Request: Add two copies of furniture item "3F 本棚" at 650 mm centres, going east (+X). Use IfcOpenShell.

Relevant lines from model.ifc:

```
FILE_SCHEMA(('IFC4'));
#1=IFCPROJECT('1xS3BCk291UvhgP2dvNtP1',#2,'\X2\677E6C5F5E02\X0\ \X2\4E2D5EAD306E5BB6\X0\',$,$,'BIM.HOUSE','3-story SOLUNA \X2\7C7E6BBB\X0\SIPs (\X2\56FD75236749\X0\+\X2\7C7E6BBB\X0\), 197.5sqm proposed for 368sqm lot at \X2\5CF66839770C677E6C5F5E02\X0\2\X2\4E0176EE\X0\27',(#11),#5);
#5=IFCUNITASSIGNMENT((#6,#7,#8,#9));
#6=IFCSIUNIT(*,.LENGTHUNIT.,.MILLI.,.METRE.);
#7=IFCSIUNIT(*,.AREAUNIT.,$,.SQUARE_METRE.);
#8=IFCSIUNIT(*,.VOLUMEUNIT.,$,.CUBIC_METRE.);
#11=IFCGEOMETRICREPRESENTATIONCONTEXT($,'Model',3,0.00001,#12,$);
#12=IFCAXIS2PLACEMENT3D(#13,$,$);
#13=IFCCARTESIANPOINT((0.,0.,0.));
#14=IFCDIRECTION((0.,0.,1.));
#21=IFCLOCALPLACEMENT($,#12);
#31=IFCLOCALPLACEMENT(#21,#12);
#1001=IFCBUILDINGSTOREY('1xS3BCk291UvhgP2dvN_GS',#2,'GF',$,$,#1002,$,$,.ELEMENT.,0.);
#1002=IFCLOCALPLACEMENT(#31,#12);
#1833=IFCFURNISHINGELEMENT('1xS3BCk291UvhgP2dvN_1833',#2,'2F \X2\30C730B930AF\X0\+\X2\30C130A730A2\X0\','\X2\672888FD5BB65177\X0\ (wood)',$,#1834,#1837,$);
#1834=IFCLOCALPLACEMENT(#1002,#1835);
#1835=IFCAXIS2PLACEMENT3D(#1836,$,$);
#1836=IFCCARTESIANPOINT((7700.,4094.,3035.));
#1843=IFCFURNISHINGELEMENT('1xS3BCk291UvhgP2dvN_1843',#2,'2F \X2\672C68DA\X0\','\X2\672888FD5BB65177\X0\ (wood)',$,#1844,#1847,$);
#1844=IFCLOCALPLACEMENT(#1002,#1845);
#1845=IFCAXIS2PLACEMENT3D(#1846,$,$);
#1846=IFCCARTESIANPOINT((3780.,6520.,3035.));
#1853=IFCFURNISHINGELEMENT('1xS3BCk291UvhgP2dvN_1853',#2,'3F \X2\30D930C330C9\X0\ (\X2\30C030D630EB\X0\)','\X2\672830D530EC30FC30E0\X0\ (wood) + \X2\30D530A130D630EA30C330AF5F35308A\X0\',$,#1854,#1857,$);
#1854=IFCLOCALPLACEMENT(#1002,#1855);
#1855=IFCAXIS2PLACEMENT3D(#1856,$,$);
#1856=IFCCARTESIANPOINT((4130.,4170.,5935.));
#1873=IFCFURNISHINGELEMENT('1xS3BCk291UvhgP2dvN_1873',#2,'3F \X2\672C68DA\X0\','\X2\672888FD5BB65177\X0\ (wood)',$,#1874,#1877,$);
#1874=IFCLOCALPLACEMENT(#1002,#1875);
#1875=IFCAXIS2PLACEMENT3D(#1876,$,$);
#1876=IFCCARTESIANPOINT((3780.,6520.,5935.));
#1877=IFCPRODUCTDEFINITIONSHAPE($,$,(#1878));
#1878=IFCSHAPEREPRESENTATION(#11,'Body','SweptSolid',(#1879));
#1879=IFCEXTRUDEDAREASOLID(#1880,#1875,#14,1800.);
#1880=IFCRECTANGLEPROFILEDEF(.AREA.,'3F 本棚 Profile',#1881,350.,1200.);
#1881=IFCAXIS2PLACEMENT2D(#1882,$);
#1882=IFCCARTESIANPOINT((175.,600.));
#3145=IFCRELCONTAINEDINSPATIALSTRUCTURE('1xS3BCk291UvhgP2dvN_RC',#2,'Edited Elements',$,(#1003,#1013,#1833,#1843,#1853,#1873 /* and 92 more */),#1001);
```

```python
import numpy as np
import ifcopenshell
import ifcopenshell.api.geometry
import ifcopenshell.api.root
import ifcopenshell.util.element
import ifcopenshell.util.placement
import ifcopenshell.util.unit

model = ifcopenshell.open("model.ifc")
unit_scale = ifcopenshell.util.unit.calculate_unit_scale(model)


def reuse_history(source, copy):
    """copy_class also copies each property set's owner history, people and application; keep the originals."""
    for rel in copy.IsDefinedBy:
        if rel.is_a("IfcRelDefinesByProperties") and (history := rel.RelatingPropertyDefinition.OwnerHistory):
            rel.RelatingPropertyDefinition.OwnerHistory = source.OwnerHistory
            ifcopenshell.util.element.remove_deep2(model, history)


source = model.by_guid("1xS3BCk291UvhgP2dvN_1873")
base = ifcopenshell.util.placement.get_local_placement(source.ObjectPlacement)
step = np.array([1.0, 0.0, 0.0]) * 0.65 / unit_scale

for i in range(1, 3):
    copy = ifcopenshell.api.root.copy_class(model, product=source)
    copy.Representation = ifcopenshell.util.element.copy_deep(
        model, source.Representation, exclude=["IfcGeometricRepresentationContext", "IfcRepresentationMap"]
    )
    reuse_history(source, copy)
    matrix = base.copy()
    matrix[:3, 3] += i * step
    print("added at", matrix[:3, 3].round(3) + 0.0)
    ifcopenshell.api.geometry.edit_object_placement(model, product=copy, matrix=matrix, is_si=False)

model.write("model_v2.ifc")
```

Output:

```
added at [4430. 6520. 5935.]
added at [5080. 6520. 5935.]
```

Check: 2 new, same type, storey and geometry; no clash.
